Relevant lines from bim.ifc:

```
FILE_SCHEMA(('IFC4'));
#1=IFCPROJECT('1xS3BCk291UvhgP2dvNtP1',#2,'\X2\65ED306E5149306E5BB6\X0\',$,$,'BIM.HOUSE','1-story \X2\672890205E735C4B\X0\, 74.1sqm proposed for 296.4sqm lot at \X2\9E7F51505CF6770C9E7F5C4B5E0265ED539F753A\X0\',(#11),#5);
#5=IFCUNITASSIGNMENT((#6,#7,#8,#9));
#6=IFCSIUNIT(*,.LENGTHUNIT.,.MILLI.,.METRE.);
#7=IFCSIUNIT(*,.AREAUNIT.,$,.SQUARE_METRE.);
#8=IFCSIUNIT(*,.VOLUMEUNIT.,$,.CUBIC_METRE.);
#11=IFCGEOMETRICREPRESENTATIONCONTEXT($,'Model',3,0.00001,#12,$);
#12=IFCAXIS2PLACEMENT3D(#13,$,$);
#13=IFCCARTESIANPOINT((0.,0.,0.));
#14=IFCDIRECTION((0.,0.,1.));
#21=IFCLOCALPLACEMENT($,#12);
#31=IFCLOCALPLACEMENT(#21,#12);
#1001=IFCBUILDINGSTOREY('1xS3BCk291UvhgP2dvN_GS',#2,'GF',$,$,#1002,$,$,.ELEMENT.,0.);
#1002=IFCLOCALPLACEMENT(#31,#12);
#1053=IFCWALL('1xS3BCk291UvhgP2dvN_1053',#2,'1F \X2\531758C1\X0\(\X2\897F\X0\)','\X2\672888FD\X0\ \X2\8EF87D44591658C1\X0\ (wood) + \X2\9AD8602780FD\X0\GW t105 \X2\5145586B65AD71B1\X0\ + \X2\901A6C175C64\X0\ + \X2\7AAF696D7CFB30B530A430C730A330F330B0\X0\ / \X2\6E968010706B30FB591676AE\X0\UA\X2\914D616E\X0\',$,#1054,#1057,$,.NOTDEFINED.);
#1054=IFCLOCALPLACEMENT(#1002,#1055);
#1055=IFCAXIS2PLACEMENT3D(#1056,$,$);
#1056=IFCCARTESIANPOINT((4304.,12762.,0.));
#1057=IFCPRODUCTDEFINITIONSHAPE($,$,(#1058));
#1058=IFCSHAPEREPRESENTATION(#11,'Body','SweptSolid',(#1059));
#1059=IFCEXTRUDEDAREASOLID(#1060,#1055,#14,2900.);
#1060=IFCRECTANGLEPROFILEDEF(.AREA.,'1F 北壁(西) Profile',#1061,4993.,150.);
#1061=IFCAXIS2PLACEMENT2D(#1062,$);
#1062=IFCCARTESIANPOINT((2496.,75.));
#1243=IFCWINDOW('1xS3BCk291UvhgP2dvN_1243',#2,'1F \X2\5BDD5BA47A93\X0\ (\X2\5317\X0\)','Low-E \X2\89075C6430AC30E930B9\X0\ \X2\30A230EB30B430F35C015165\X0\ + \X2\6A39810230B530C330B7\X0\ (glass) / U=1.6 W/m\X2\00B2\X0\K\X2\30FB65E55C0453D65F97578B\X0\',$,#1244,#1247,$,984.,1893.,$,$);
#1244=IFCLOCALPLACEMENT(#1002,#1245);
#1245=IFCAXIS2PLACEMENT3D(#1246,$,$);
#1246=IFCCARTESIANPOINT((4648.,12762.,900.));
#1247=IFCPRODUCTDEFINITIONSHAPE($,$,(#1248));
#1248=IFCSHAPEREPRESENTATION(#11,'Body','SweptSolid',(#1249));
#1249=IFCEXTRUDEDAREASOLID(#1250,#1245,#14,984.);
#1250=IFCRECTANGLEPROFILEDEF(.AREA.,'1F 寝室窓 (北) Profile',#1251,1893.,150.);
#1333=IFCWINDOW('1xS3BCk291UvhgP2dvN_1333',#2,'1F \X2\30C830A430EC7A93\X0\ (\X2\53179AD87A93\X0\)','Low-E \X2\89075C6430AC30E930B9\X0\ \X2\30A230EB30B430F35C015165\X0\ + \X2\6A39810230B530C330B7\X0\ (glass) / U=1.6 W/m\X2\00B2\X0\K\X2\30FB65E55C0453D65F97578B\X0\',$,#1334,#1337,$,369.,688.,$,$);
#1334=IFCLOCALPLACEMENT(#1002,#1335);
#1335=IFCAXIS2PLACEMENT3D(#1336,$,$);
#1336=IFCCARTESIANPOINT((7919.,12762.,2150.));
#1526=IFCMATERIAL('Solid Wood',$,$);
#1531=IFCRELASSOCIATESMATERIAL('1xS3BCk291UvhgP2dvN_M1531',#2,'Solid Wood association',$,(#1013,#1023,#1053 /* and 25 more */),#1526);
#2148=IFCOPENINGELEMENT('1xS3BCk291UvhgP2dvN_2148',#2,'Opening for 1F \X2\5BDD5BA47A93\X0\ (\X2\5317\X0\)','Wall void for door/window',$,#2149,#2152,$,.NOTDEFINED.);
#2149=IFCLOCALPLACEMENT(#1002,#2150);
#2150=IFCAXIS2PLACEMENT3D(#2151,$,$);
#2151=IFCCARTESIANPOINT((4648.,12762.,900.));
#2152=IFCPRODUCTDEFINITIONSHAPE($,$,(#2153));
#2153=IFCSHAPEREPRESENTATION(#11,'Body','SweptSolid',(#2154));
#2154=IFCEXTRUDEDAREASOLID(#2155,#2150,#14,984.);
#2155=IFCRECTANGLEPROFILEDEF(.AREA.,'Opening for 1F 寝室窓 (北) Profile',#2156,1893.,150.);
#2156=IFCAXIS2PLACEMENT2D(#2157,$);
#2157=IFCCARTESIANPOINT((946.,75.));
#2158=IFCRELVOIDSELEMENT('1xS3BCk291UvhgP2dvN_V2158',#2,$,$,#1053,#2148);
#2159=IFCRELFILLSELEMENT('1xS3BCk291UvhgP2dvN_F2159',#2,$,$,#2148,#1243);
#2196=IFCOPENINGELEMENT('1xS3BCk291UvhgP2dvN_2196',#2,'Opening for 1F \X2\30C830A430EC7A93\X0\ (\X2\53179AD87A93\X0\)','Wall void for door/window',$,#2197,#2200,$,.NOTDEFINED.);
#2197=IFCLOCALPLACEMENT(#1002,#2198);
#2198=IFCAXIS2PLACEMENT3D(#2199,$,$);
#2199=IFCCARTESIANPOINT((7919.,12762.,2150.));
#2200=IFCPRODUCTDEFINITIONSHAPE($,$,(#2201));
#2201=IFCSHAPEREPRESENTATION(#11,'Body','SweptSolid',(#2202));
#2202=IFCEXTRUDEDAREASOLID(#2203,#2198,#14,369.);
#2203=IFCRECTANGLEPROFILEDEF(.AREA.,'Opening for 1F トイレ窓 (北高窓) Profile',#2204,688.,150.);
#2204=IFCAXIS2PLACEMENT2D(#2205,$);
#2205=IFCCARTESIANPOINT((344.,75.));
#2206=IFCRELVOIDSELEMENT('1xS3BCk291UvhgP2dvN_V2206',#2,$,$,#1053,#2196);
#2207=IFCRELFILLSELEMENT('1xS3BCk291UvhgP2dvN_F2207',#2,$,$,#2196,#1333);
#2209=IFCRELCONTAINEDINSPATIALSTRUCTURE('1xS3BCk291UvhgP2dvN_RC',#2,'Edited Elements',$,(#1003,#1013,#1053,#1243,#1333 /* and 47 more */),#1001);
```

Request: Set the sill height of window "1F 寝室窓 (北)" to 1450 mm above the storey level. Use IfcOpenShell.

```python
import numpy as np
import ifcopenshell
import ifcopenshell.api.geometry
import ifcopenshell.geom
import ifcopenshell.util.element
import ifcopenshell.util.placement
import ifcopenshell.util.shape
import ifcopenshell.util.unit

model = ifcopenshell.open("bim.ifc")
unit_scale = ifcopenshell.util.unit.calculate_unit_scale(model)

window = model.by_guid("1xS3BCk291UvhgP2dvN_1243")
opening = window.FillsVoids[0].RelatingOpeningElement
storey = ifcopenshell.util.element.get_container(window, ifc_class="IfcBuildingStorey")
level = ifcopenshell.util.placement.get_local_placement(storey.ObjectPlacement)[2, 3]

# The opening's origin need not be at the sill, so measure its lowest point.
shape = ifcopenshell.geom.create_shape(ifcopenshell.geom.settings(), opening)
bottom = ifcopenshell.util.shape.get_shape_bottom_elevation(shape, shape.geometry) / unit_scale
dz = level + 1.45 / unit_scale - bottom

shift = np.array([0.0, 0.0, dz])
# The window is not placed relative to its opening, so move both.
for product in (opening, window):
    matrix = ifcopenshell.util.placement.get_local_placement(product.ObjectPlacement)
    matrix[:3, 3] += shift
    ifcopenshell.api.geometry.edit_object_placement(model, product=product, matrix=matrix, is_si=False)

print(f"moved by {dz * unit_scale:+.3f} m")

model.write("bim-out.ifc")
```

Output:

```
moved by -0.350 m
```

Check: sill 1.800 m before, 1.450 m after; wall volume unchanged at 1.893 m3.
